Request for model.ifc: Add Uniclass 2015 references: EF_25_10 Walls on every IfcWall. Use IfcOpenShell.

First a look at what the model holds.

```python
import ifcopenshell

model = ifcopenshell.open("model.ifc")
print(model.schema)
print("classifications:", [c.Name for c in model.by_type("IfcClassification")])
for ifc_class in ("IfcDoor", "IfcRoof", "IfcStair", "IfcWall", "IfcWindow"):
    print(ifc_class, len(model.by_type(ifc_class)))
```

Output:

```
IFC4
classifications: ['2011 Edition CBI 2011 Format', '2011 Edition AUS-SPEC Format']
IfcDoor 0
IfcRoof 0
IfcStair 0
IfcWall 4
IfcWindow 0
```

```python
import ifcopenshell
import ifcopenshell.api.classification

model = ifcopenshell.open("model.ifc")

system = ifcopenshell.api.classification.add_classification(model, classification="Uniclass 2015")

codes = {
    "IfcWall": ("EF_25_10", "Walls"),
}
for ifc_class, (code, name) in codes.items():
    products = model.by_type(ifc_class)
    ifcopenshell.api.classification.add_reference(
        model, products=products, classification=system, identification=code, name=name
    )
    print(code, len(products))

model.write("model_edited.ifc")
```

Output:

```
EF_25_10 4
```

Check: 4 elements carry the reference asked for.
